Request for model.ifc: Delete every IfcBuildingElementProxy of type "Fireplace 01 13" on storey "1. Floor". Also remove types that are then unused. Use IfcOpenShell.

First a look at what the model holds.

```python
import ifcopenshell
import ifcopenshell.util.element

model = ifcopenshell.open("model.ifc")
print(model.schema)
storey = next(s for s in model.by_type("IfcBuildingStorey") if s.Name == "1. Floor")
proxies = [e for e in ifcopenshell.util.element.get_decomposition(storey) if e.is_a("IfcBuildingElementProxy")]
seen = {}
for e in proxies:
    element_type = ifcopenshell.util.element.get_type(e)
    name = element_type.Name if element_type not in (None, e) else None
    seen[name] = seen.get(name, 0) + 1
for name, count in sorted(seen.items(), key=str):
    print(count, "x", name)
```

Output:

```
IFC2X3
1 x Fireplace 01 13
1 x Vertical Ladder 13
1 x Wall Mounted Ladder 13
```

```python
import ifcopenshell
import ifcopenshell.api.root
import ifcopenshell.util.element

model = ifcopenshell.open("model.ifc")

storey = next(s for s in model.by_type("IfcBuildingStorey") if s.Name == "1. Floor")
proxies = [e for e in ifcopenshell.util.element.get_decomposition(storey) if e.is_a("IfcBuildingElementProxy")]
targets = [e for e in proxies if (t := ifcopenshell.util.element.get_type(e)) not in (None, e) and t.Name == "Fireplace 01 13"]
types = {ifcopenshell.util.element.get_type(e) for e in targets} - {None, *targets}

for e in targets:
    ifcopenshell.api.root.remove_product(model, product=e)
print(len(targets), "removed")

unused = [t for t in types if not ifcopenshell.util.element.get_types(t)]
for t in unused:
    ifcopenshell.api.root.remove_product(model, product=t)
print(len(unused), "unused types removed")

model.write("model-out.ifc")
```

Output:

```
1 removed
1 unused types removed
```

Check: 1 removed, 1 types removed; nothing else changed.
